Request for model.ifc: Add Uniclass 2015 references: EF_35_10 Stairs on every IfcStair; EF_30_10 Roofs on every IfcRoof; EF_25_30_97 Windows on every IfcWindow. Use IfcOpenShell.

First a look at what the model holds.

```python
import ifcopenshell

model = ifcopenshell.open("model.ifc")
print(model.schema)
print("classifications:", [c.Name for c in model.by_type("IfcClassification")])
for ifc_class in ("IfcDoor", "IfcRoof", "IfcStair", "IfcWall", "IfcWindow"):
    print(ifc_class, len(model.by_type(ifc_class)))
```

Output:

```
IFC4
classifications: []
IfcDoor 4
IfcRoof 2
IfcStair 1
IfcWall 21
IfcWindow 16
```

```python
import ifcopenshell
import ifcopenshell.api.classification

model = ifcopenshell.open("model.ifc")

system = ifcopenshell.api.classification.add_classification(model, classification="Uniclass 2015")

codes = {
    "IfcStair": ("EF_35_10", "Stairs"),
    "IfcRoof": ("EF_30_10", "Roofs"),
    "IfcWindow": ("EF_25_30_97", "Windows"),
}
for ifc_class, (code, name) in codes.items():
    products = model.by_type(ifc_class)
    ifcopenshell.api.classification.add_reference(
        model, products=products, classification=system, identification=code, name=name
    )
    print(code, len(products))

model.write("model_v2.ifc")
```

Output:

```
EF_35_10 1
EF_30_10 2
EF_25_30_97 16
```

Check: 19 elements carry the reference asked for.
